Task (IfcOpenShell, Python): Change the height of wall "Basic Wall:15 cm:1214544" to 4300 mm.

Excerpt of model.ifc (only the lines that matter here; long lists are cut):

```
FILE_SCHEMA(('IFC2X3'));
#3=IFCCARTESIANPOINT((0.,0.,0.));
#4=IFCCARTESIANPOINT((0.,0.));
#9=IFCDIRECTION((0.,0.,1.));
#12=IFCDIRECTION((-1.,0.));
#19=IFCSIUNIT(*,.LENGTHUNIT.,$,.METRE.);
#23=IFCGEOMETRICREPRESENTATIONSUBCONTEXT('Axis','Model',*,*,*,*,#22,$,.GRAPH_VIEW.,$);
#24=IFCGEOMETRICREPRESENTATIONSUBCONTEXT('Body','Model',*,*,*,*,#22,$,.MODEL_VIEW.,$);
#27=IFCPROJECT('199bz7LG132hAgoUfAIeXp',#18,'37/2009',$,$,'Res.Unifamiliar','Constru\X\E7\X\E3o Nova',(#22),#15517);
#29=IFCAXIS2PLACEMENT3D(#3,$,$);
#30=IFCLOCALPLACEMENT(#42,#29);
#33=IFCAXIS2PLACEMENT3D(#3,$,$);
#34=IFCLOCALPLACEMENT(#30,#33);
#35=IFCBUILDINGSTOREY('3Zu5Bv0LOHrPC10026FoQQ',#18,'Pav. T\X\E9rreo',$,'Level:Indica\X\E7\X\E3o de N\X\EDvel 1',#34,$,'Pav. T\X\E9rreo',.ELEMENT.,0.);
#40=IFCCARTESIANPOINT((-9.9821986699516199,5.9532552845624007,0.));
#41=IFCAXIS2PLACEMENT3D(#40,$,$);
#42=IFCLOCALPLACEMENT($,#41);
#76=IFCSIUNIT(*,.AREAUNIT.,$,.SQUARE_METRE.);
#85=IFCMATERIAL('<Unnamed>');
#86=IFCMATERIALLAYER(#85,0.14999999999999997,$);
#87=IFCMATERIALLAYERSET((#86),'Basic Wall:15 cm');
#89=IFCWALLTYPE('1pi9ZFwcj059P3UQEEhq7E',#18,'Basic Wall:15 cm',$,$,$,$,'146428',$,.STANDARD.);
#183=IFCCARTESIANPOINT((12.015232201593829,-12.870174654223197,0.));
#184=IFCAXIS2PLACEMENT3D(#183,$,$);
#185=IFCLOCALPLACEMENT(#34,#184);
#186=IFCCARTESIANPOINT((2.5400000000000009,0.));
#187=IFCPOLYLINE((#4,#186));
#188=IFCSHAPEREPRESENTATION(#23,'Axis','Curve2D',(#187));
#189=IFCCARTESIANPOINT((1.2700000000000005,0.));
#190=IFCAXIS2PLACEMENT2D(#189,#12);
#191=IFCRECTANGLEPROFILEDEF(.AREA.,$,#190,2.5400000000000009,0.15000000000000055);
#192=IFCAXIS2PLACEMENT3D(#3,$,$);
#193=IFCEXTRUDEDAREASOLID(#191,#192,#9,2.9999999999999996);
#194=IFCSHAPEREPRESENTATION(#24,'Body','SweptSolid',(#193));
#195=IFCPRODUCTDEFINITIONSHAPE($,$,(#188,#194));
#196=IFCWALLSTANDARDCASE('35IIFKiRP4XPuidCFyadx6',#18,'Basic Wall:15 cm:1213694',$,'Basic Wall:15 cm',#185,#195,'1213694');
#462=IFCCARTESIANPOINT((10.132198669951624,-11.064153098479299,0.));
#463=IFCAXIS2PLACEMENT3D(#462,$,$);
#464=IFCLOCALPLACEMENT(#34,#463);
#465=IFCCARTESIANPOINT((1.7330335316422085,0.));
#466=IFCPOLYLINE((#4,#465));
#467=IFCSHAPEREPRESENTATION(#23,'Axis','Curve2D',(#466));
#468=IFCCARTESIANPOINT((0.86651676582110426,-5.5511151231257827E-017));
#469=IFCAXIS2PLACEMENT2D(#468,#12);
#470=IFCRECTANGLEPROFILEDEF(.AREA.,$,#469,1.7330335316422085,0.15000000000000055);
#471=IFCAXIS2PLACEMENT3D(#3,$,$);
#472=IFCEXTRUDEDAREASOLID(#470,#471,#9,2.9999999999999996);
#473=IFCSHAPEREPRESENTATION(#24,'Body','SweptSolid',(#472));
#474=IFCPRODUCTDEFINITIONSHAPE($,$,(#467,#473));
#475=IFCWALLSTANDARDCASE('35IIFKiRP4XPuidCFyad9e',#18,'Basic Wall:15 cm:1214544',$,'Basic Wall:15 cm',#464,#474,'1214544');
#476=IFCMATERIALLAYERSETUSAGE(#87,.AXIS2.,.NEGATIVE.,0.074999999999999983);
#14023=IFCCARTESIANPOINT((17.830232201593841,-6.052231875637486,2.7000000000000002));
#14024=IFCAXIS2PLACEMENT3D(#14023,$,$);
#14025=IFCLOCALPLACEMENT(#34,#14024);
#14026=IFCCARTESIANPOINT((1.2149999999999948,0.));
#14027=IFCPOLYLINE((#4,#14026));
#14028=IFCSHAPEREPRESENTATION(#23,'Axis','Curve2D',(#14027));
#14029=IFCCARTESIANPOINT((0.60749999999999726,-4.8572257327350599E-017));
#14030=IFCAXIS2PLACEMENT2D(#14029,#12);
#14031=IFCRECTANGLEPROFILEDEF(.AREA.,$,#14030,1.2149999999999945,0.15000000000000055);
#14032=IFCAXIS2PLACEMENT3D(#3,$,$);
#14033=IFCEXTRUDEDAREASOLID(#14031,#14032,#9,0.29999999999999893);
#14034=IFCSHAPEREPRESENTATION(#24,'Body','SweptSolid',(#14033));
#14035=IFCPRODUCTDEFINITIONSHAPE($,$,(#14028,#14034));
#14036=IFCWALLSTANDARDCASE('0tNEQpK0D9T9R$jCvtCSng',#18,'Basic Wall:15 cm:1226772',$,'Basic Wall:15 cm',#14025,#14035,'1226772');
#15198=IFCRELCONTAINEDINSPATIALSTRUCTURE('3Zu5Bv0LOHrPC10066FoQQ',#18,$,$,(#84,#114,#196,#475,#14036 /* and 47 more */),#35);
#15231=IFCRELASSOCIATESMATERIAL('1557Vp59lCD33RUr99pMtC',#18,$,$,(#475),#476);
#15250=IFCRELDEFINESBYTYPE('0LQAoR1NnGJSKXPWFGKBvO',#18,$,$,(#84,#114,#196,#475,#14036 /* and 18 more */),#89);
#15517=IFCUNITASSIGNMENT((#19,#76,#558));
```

```python
import ifcopenshell
import ifcopenshell.geom
import ifcopenshell.util.representation
import ifcopenshell.util.shape

model = ifcopenshell.open("model.ifc")
settings = ifcopenshell.geom.settings()


def volume(element):
    """Net volume in cubic metres, openings subtracted."""
    shape = ifcopenshell.geom.create_shape(settings, element)
    return ifcopenshell.util.shape.get_volume(shape.geometry)


wall = model.by_guid("35IIFKiRP4XPuidCFyad9e")
before = volume(wall)

body = ifcopenshell.util.representation.get_representation(wall, "Model", "Body")
solid = body.Items[0]
old_height = solid.Depth
solid.Depth = 4.3
after = volume(wall)

print(f"height {old_height:g} -> {solid.Depth:g}, volume {before:.3f} -> {after:.3f} m3")

model.write("model_updated.ifc")
```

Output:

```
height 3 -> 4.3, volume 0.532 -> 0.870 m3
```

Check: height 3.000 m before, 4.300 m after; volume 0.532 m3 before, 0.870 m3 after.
